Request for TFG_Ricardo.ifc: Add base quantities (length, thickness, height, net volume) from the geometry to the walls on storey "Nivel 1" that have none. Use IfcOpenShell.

First a look at what the model holds.

```python
import ifcopenshell
import ifcopenshell.util.element
import ifcopenshell.util.unit

model = ifcopenshell.open("TFG_Ricardo.ifc")
print(model.schema)
for unit_type in ("LENGTHUNIT", "AREAUNIT", "VOLUMEUNIT"):
    print(unit_type, ifcopenshell.util.unit.calculate_unit_scale(model, unit_type))
storey = next(s for s in model.by_type("IfcBuildingStorey") if s.Name == "Nivel 1")
walls = [e for e in ifcopenshell.util.element.get_decomposition(storey) if e.is_a("IfcWall")]
for e in sorted(walls, key=lambda e: e.id()):
    print(e.id(), e.is_a(), e.Name, list(ifcopenshell.util.element.get_psets(e, qtos_only=True)), sep=" | ")
```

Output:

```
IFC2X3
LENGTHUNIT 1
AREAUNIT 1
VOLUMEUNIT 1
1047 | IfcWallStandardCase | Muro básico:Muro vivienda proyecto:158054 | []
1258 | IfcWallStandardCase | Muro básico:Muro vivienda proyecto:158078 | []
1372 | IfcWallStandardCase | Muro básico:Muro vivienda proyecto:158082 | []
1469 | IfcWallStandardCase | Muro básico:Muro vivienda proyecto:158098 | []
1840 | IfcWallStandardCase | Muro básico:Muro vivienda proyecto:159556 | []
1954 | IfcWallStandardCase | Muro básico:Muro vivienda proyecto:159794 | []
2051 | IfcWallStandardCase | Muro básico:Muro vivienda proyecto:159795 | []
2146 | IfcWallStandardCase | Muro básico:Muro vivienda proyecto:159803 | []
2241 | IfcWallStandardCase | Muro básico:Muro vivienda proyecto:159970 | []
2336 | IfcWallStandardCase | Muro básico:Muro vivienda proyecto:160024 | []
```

```python
import ifcopenshell
import ifcopenshell.api.pset
import ifcopenshell.geom
import ifcopenshell.util.element
import ifcopenshell.util.shape
import ifcopenshell.util.unit

model = ifcopenshell.open("TFG_Ricardo.ifc")
unit_scale = ifcopenshell.util.unit.calculate_unit_scale(model)
volume_scale = ifcopenshell.util.unit.calculate_unit_scale(model, "VOLUMEUNIT")
settings = ifcopenshell.geom.settings()

storey = next(s for s in model.by_type("IfcBuildingStorey") if s.Name == "Nivel 1")
walls = [e for e in ifcopenshell.util.element.get_decomposition(storey) if e.is_a("IfcWall")]

for e in sorted(walls, key=lambda e: e.id()):
    if ifcopenshell.util.element.get_psets(e, qtos_only=True, should_inherit=False):
        continue
    # Geometry comes back in metres, in the element's own axes.
    shape = ifcopenshell.geom.create_shape(settings, e)
    values = {
        "Length": ifcopenshell.util.shape.get_x(shape.geometry) / unit_scale,
        "Width": ifcopenshell.util.shape.get_y(shape.geometry) / unit_scale,
        "Height": ifcopenshell.util.shape.get_z(shape.geometry) / unit_scale,
        "NetVolume": ifcopenshell.util.shape.get_volume(shape.geometry) / volume_scale,
    }
    qto = ifcopenshell.api.pset.add_qto(model, product=e, name="BaseQuantities")
    ifcopenshell.api.pset.edit_qto(model, qto=qto, properties=values)
    print(e.id(), {k: round(v, 3) for k, v in values.items()})

model.write("TFG_Ricardo-out.ifc")
```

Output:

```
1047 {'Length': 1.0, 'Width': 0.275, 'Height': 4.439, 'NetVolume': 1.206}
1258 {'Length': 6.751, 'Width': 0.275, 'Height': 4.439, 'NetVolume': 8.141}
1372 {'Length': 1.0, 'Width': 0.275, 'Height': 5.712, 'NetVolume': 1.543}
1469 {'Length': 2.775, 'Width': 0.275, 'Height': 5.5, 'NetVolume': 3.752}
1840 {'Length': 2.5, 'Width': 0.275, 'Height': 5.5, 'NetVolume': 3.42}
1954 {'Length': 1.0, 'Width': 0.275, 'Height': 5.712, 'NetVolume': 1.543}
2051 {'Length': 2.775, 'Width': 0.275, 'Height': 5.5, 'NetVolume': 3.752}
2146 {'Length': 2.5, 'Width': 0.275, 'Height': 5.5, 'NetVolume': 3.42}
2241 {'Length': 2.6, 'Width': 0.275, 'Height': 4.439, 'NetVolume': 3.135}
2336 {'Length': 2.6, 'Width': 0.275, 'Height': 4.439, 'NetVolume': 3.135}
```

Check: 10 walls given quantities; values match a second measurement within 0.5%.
